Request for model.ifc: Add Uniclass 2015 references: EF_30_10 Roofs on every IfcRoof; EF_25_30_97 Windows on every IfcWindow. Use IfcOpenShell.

First a look at what the model holds.

```python
import ifcopenshell

model = ifcopenshell.open("model.ifc")
print(model.schema)
print("classifications:", [c.Name for c in model.by_type("IfcClassification")])
for ifc_class in ("IfcDoor", "IfcRoof", "IfcStair", "IfcWall", "IfcWindow"):
    print(ifc_class, len(model.by_type(ifc_class)))
```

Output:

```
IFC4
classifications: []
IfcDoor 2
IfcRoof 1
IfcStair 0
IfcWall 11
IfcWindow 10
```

```python
import ifcopenshell
import ifcopenshell.api.classification

model = ifcopenshell.open("model.ifc")

system = ifcopenshell.api.classification.add_classification(model, classification="Uniclass 2015")

codes = {
    "IfcRoof": ("EF_30_10", "Roofs"),
    "IfcWindow": ("EF_25_30_97", "Windows"),
}
for ifc_class, (code, name) in codes.items():
    products = model.by_type(ifc_class)
    ifcopenshell.api.classification.add_reference(
        model, products=products, classification=system, identification=code, name=name
    )
    print(code, len(products))

model.write("model_rev.ifc")
```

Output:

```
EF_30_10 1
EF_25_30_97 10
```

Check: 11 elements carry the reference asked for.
